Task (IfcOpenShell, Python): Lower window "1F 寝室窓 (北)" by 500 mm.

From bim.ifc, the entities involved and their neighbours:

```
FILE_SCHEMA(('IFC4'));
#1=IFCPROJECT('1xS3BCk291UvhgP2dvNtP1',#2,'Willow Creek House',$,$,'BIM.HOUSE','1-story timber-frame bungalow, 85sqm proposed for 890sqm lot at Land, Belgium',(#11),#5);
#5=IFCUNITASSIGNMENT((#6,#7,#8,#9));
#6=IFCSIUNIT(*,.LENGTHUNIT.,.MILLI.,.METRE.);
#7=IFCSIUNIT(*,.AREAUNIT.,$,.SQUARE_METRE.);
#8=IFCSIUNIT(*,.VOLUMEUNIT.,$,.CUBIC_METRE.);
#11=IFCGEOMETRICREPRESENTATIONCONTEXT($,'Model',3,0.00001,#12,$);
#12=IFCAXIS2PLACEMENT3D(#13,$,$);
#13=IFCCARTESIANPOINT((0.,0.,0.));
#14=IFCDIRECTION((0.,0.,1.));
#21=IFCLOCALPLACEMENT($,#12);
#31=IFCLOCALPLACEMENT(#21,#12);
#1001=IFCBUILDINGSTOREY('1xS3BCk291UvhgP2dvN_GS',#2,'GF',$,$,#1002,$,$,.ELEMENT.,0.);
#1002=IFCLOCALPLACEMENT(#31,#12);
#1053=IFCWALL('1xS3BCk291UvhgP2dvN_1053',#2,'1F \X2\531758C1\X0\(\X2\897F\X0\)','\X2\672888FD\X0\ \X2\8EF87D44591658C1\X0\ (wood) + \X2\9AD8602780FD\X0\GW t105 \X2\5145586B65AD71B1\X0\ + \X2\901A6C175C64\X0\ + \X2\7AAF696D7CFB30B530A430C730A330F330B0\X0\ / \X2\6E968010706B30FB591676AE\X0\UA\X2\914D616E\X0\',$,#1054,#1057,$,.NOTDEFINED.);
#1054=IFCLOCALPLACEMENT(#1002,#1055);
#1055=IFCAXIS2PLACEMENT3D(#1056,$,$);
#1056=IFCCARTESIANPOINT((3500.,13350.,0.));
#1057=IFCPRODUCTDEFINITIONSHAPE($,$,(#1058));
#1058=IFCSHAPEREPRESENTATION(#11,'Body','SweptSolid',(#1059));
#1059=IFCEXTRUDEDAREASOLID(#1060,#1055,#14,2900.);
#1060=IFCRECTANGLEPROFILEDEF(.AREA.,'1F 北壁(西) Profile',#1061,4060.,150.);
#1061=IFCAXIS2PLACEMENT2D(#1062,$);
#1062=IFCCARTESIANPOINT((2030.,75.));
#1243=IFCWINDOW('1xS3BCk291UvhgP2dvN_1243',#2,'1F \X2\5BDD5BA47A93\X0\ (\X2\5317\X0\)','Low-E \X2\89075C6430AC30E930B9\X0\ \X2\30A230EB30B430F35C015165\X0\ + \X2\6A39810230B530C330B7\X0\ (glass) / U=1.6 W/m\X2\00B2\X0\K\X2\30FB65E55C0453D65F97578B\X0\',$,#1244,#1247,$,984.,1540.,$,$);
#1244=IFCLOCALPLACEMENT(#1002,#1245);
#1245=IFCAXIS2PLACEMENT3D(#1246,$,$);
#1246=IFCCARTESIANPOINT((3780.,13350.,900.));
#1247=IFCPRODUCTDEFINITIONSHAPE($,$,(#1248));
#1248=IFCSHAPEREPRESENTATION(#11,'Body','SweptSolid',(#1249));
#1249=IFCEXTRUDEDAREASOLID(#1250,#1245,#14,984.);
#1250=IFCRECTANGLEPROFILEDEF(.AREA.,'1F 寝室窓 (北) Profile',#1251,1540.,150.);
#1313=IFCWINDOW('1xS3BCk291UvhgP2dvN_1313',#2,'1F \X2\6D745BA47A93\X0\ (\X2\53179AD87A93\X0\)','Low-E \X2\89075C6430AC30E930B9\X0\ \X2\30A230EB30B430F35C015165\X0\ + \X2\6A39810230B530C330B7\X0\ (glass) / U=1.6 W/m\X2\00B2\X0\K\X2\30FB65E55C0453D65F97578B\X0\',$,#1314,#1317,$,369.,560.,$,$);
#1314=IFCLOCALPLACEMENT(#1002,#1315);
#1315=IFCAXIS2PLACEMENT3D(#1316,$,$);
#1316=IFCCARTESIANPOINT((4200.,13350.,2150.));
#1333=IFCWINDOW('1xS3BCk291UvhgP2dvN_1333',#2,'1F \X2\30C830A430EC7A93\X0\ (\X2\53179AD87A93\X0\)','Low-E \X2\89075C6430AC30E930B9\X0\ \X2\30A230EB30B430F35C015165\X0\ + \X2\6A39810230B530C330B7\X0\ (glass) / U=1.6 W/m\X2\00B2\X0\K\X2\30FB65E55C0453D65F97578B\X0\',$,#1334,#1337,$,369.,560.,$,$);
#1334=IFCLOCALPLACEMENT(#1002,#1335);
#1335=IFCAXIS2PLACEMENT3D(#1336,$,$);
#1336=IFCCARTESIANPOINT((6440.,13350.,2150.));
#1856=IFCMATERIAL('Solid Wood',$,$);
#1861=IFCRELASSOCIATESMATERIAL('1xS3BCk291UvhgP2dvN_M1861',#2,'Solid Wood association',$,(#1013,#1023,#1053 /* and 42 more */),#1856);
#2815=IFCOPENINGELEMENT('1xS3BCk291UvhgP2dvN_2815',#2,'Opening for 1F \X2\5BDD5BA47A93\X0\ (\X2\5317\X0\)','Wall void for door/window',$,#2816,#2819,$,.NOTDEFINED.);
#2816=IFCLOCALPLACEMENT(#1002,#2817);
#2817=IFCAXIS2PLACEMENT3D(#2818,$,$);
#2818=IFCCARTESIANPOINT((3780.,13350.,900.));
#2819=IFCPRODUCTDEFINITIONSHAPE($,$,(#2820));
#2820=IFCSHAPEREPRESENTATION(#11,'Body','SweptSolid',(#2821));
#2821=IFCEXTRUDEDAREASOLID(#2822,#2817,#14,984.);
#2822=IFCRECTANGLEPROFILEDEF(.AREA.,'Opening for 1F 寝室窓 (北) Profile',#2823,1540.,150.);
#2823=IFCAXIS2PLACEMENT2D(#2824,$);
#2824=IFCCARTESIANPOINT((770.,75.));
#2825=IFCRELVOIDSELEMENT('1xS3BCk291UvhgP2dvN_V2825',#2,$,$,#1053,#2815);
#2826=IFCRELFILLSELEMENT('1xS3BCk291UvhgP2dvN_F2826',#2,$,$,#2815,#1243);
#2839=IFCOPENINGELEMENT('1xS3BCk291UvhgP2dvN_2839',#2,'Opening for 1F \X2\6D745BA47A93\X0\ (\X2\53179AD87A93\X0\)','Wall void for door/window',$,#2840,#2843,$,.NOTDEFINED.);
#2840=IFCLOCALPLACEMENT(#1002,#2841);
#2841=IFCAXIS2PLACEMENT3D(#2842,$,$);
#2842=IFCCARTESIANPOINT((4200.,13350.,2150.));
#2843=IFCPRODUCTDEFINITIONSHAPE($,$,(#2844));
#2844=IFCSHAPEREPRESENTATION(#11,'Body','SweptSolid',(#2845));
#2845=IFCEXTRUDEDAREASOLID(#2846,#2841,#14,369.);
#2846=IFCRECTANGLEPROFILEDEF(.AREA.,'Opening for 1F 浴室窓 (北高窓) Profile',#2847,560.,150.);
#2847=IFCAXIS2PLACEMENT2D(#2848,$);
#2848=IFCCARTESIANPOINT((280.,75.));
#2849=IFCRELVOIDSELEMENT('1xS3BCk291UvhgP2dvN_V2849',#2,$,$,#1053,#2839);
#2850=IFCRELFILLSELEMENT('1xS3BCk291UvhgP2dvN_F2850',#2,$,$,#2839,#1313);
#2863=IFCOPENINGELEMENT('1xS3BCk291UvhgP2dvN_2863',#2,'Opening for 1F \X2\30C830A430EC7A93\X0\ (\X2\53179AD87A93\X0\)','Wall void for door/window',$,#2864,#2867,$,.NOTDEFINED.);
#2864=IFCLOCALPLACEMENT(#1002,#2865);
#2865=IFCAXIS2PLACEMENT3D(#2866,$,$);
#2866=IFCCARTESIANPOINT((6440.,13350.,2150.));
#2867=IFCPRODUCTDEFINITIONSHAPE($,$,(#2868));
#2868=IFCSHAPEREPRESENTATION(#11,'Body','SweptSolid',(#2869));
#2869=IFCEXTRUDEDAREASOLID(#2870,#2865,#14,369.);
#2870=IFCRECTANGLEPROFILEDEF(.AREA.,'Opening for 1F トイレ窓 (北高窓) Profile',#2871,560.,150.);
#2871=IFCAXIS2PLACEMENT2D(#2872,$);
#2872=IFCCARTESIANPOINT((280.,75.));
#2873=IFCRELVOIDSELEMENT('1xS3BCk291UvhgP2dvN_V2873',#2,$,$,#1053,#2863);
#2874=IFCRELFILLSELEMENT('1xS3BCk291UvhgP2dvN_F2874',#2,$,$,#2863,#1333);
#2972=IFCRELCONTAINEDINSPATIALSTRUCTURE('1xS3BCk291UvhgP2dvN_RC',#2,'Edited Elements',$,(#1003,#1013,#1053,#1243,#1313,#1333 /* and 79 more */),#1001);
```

```python
import numpy as np
import ifcopenshell
import ifcopenshell.api.geometry
import ifcopenshell.util.placement
import ifcopenshell.util.unit

model = ifcopenshell.open("bim.ifc")
unit_scale = ifcopenshell.util.unit.calculate_unit_scale(model)

window = model.by_guid("1xS3BCk291UvhgP2dvN_1243")
opening = window.FillsVoids[0].RelatingOpeningElement
dz = -0.5 / unit_scale

shift = np.array([0.0, 0.0, dz])
# The window is not placed relative to its opening, so move both.
for product in (opening, window):
    matrix = ifcopenshell.util.placement.get_local_placement(product.ObjectPlacement)
    matrix[:3, 3] += shift
    ifcopenshell.api.geometry.edit_object_placement(model, product=product, matrix=matrix, is_si=False)

print(f"moved by {dz * unit_scale:+.3f} m")

model.write("bim_updated.ifc")
```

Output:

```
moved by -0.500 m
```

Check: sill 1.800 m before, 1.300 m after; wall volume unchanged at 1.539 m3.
